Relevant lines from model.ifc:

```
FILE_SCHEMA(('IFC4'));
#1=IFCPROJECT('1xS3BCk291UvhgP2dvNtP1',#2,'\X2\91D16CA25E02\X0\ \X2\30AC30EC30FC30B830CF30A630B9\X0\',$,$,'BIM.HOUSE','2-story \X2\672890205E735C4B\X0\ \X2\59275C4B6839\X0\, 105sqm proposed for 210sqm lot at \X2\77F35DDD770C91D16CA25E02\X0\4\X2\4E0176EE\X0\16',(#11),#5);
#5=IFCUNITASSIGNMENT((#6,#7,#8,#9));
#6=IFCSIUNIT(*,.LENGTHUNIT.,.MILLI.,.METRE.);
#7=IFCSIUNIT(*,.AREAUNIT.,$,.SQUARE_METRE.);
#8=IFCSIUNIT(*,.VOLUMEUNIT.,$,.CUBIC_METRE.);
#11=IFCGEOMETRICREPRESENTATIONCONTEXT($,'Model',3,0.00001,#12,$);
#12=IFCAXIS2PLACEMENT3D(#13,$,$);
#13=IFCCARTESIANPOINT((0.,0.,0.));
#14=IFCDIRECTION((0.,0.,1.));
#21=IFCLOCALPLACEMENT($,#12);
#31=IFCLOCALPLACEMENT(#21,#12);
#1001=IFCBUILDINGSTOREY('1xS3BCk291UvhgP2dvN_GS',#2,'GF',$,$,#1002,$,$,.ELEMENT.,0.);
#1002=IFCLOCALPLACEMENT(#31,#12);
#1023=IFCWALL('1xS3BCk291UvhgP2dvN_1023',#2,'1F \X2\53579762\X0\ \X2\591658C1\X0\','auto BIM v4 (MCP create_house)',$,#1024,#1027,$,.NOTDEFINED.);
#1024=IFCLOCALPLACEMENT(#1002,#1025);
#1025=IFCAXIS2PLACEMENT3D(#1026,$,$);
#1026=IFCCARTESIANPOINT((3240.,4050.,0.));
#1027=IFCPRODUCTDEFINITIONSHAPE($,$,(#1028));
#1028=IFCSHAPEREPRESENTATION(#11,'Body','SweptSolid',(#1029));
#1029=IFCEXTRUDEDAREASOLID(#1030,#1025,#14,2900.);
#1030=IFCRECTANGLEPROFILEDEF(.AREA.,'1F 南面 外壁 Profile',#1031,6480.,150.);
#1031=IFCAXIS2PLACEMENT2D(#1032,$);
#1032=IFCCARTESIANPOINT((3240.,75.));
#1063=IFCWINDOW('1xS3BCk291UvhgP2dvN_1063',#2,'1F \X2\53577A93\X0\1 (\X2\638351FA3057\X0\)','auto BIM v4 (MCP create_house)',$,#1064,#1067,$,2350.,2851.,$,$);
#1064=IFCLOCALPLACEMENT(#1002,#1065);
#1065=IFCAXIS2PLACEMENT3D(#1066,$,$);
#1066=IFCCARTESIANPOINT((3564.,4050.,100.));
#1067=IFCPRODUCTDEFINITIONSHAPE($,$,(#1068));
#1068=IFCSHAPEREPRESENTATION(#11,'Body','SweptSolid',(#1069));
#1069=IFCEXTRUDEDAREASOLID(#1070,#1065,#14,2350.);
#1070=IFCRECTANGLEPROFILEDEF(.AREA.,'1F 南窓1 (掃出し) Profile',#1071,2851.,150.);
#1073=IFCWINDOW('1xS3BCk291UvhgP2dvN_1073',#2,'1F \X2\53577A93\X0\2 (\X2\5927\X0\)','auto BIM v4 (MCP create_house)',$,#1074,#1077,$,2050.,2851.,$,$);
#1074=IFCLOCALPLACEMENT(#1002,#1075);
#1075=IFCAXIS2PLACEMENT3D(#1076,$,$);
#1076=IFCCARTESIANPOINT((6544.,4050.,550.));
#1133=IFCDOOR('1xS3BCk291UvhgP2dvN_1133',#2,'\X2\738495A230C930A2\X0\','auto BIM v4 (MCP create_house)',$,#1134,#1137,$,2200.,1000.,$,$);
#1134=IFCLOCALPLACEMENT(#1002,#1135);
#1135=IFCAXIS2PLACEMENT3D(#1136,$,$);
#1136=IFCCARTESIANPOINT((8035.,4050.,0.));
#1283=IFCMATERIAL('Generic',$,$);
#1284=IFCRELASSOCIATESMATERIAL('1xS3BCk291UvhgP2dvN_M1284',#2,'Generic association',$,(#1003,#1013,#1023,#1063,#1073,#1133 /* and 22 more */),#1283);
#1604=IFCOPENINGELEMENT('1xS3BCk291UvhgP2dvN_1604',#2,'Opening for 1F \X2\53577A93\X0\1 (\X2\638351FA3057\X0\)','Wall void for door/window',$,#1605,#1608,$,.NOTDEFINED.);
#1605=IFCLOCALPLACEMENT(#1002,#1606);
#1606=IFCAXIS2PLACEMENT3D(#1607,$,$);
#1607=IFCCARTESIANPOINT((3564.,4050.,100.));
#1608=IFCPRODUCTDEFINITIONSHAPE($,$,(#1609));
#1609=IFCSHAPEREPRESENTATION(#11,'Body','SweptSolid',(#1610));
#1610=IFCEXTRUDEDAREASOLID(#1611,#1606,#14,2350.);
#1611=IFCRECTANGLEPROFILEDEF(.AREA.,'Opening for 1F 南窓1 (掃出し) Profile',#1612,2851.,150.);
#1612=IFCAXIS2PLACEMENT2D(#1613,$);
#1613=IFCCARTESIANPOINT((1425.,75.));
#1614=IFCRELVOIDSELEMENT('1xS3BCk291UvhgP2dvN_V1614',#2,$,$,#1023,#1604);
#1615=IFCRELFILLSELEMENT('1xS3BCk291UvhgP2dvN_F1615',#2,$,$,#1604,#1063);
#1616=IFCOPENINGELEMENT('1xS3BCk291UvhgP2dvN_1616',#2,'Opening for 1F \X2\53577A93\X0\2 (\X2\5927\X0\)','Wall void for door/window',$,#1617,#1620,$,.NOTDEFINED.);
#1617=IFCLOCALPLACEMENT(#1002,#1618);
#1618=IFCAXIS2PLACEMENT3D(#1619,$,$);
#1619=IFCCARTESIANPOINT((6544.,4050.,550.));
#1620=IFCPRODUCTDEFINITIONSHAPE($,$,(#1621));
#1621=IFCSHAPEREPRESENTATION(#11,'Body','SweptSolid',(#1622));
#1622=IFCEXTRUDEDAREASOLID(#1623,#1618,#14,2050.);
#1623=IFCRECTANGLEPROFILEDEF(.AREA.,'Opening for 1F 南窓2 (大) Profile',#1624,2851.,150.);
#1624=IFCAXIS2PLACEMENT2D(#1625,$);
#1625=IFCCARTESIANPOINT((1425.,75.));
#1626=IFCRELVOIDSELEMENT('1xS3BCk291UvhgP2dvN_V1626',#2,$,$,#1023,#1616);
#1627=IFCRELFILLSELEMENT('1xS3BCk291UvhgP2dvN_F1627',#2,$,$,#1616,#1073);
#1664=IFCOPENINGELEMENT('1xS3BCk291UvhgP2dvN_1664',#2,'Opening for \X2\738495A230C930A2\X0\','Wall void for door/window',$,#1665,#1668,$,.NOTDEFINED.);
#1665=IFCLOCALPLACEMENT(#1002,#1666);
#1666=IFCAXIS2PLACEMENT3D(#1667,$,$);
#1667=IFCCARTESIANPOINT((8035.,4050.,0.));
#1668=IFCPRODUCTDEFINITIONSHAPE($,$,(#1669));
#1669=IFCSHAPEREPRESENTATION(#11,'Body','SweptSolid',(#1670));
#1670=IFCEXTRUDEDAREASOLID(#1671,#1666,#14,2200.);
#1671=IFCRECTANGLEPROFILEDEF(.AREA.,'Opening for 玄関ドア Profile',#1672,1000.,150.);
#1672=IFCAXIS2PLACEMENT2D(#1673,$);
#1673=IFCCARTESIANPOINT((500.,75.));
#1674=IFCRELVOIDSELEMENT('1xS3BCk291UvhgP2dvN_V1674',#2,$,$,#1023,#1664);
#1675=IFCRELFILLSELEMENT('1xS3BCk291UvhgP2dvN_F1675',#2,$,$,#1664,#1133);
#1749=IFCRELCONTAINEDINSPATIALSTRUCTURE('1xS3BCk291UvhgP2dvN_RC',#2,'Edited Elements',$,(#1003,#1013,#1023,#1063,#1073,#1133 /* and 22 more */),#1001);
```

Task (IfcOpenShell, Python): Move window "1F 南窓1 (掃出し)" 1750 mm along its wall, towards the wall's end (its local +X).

```python
import ifcopenshell
import ifcopenshell.api.geometry
import ifcopenshell.util.placement
import ifcopenshell.util.unit

model = ifcopenshell.open("model.ifc")
unit_scale = ifcopenshell.util.unit.calculate_unit_scale(model)

window = model.by_guid("1xS3BCk291UvhgP2dvN_1063")
opening = window.FillsVoids[0].RelatingOpeningElement
wall = opening.VoidsElements[0].RelatingBuildingElement

wall_matrix = ifcopenshell.util.placement.get_local_placement(wall.ObjectPlacement)
shift = wall_matrix[:3, 0] * 1.75 / unit_scale
before = ifcopenshell.util.placement.get_local_placement(window.ObjectPlacement)[:3, 3].copy()

# The window is not placed relative to its opening, so move both.
for product in (opening, window):
    matrix = ifcopenshell.util.placement.get_local_placement(product.ObjectPlacement)
    matrix[:3, 3] += shift
    ifcopenshell.api.geometry.edit_object_placement(model, product=product, matrix=matrix, is_si=False)

after = ifcopenshell.util.placement.get_local_placement(window.ObjectPlacement)[:3, 3]
print("window moved by", (after - before).round(3) + 0.0)

model.write("model_rev.ifc")
```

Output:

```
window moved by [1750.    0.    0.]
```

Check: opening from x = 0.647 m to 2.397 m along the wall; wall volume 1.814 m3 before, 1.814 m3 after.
